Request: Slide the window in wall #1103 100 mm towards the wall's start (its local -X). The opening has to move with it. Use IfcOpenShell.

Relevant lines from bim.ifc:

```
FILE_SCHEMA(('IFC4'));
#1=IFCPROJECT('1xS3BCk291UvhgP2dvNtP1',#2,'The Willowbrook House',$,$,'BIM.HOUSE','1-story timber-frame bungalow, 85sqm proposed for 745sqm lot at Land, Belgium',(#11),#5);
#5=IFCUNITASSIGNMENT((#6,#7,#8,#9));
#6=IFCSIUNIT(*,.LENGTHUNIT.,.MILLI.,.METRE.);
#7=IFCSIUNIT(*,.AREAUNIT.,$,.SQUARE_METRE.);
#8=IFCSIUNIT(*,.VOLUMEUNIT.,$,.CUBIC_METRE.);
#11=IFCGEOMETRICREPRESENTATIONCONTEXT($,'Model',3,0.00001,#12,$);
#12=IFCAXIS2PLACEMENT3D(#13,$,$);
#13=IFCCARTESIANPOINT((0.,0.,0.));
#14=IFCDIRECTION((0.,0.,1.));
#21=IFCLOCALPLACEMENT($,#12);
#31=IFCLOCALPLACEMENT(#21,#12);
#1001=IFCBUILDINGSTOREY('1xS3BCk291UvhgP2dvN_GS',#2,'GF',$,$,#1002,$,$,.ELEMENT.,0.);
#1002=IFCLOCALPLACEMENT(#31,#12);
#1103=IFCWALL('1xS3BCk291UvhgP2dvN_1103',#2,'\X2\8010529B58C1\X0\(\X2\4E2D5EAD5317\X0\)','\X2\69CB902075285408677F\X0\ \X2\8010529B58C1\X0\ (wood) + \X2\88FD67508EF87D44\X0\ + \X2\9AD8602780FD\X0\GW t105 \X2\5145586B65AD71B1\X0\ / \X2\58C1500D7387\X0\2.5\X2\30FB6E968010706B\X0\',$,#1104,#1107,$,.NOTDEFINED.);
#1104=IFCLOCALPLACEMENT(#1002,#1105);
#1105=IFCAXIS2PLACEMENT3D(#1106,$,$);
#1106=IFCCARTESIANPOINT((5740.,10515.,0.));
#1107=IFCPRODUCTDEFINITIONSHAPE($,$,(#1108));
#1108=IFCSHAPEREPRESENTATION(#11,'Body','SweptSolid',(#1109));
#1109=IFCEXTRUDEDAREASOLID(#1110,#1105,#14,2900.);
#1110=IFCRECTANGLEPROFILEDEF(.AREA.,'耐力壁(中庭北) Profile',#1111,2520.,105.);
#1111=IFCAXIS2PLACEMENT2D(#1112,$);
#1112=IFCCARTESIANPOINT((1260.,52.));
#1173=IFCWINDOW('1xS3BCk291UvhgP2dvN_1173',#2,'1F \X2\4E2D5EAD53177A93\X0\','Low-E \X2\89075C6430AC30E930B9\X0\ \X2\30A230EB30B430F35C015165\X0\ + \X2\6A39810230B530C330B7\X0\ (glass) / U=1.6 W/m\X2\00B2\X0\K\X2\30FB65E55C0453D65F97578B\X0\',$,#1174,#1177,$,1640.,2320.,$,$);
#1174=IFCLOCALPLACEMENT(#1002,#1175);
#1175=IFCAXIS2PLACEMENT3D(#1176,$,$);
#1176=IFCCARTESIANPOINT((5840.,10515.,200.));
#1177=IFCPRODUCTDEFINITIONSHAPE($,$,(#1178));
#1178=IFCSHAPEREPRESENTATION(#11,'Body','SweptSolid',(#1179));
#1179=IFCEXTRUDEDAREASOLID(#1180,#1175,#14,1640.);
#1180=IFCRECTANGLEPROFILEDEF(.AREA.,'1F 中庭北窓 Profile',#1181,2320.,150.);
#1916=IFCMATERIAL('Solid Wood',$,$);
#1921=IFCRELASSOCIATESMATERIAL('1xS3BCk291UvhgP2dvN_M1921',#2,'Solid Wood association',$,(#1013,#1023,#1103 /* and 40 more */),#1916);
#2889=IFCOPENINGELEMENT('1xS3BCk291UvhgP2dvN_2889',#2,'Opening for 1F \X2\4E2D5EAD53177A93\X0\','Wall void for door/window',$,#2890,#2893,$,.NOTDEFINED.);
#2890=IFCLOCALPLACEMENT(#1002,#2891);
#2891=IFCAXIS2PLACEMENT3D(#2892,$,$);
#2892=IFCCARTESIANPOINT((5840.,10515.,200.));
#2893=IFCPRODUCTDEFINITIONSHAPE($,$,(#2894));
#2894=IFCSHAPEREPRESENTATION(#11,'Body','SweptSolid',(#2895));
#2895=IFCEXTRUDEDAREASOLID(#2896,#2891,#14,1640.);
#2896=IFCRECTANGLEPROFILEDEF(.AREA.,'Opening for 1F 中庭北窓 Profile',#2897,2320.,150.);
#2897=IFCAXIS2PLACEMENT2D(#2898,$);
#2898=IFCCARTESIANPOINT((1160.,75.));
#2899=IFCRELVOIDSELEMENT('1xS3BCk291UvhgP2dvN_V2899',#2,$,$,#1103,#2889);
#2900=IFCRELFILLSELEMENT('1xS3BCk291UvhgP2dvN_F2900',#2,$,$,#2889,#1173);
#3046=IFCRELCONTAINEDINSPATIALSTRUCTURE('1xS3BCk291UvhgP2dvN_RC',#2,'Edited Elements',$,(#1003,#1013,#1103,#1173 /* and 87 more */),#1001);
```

```python
import ifcopenshell
import ifcopenshell.api.geometry
import ifcopenshell.util.placement
import ifcopenshell.util.unit

model = ifcopenshell.open("bim.ifc")
unit_scale = ifcopenshell.util.unit.calculate_unit_scale(model)

window = model.by_guid("1xS3BCk291UvhgP2dvN_1173")
opening = window.FillsVoids[0].RelatingOpeningElement
wall = opening.VoidsElements[0].RelatingBuildingElement

wall_matrix = ifcopenshell.util.placement.get_local_placement(wall.ObjectPlacement)
shift = wall_matrix[:3, 0] * -0.1 / unit_scale
before = ifcopenshell.util.placement.get_local_placement(window.ObjectPlacement)[:3, 3].copy()

# The window is not placed relative to its opening, so move both.
for product in (opening, window):
    matrix = ifcopenshell.util.placement.get_local_placement(product.ObjectPlacement)
    matrix[:3, 3] += shift
    ifcopenshell.api.geometry.edit_object_placement(model, product=product, matrix=matrix, is_si=False)

after = ifcopenshell.util.placement.get_local_placement(window.ObjectPlacement)[:3, 3]
print("window moved by", (after - before).round(3) + 0.0)

model.write("bim_v2.ifc")
```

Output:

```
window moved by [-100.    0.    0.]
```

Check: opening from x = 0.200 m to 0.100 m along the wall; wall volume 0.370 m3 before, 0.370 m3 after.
